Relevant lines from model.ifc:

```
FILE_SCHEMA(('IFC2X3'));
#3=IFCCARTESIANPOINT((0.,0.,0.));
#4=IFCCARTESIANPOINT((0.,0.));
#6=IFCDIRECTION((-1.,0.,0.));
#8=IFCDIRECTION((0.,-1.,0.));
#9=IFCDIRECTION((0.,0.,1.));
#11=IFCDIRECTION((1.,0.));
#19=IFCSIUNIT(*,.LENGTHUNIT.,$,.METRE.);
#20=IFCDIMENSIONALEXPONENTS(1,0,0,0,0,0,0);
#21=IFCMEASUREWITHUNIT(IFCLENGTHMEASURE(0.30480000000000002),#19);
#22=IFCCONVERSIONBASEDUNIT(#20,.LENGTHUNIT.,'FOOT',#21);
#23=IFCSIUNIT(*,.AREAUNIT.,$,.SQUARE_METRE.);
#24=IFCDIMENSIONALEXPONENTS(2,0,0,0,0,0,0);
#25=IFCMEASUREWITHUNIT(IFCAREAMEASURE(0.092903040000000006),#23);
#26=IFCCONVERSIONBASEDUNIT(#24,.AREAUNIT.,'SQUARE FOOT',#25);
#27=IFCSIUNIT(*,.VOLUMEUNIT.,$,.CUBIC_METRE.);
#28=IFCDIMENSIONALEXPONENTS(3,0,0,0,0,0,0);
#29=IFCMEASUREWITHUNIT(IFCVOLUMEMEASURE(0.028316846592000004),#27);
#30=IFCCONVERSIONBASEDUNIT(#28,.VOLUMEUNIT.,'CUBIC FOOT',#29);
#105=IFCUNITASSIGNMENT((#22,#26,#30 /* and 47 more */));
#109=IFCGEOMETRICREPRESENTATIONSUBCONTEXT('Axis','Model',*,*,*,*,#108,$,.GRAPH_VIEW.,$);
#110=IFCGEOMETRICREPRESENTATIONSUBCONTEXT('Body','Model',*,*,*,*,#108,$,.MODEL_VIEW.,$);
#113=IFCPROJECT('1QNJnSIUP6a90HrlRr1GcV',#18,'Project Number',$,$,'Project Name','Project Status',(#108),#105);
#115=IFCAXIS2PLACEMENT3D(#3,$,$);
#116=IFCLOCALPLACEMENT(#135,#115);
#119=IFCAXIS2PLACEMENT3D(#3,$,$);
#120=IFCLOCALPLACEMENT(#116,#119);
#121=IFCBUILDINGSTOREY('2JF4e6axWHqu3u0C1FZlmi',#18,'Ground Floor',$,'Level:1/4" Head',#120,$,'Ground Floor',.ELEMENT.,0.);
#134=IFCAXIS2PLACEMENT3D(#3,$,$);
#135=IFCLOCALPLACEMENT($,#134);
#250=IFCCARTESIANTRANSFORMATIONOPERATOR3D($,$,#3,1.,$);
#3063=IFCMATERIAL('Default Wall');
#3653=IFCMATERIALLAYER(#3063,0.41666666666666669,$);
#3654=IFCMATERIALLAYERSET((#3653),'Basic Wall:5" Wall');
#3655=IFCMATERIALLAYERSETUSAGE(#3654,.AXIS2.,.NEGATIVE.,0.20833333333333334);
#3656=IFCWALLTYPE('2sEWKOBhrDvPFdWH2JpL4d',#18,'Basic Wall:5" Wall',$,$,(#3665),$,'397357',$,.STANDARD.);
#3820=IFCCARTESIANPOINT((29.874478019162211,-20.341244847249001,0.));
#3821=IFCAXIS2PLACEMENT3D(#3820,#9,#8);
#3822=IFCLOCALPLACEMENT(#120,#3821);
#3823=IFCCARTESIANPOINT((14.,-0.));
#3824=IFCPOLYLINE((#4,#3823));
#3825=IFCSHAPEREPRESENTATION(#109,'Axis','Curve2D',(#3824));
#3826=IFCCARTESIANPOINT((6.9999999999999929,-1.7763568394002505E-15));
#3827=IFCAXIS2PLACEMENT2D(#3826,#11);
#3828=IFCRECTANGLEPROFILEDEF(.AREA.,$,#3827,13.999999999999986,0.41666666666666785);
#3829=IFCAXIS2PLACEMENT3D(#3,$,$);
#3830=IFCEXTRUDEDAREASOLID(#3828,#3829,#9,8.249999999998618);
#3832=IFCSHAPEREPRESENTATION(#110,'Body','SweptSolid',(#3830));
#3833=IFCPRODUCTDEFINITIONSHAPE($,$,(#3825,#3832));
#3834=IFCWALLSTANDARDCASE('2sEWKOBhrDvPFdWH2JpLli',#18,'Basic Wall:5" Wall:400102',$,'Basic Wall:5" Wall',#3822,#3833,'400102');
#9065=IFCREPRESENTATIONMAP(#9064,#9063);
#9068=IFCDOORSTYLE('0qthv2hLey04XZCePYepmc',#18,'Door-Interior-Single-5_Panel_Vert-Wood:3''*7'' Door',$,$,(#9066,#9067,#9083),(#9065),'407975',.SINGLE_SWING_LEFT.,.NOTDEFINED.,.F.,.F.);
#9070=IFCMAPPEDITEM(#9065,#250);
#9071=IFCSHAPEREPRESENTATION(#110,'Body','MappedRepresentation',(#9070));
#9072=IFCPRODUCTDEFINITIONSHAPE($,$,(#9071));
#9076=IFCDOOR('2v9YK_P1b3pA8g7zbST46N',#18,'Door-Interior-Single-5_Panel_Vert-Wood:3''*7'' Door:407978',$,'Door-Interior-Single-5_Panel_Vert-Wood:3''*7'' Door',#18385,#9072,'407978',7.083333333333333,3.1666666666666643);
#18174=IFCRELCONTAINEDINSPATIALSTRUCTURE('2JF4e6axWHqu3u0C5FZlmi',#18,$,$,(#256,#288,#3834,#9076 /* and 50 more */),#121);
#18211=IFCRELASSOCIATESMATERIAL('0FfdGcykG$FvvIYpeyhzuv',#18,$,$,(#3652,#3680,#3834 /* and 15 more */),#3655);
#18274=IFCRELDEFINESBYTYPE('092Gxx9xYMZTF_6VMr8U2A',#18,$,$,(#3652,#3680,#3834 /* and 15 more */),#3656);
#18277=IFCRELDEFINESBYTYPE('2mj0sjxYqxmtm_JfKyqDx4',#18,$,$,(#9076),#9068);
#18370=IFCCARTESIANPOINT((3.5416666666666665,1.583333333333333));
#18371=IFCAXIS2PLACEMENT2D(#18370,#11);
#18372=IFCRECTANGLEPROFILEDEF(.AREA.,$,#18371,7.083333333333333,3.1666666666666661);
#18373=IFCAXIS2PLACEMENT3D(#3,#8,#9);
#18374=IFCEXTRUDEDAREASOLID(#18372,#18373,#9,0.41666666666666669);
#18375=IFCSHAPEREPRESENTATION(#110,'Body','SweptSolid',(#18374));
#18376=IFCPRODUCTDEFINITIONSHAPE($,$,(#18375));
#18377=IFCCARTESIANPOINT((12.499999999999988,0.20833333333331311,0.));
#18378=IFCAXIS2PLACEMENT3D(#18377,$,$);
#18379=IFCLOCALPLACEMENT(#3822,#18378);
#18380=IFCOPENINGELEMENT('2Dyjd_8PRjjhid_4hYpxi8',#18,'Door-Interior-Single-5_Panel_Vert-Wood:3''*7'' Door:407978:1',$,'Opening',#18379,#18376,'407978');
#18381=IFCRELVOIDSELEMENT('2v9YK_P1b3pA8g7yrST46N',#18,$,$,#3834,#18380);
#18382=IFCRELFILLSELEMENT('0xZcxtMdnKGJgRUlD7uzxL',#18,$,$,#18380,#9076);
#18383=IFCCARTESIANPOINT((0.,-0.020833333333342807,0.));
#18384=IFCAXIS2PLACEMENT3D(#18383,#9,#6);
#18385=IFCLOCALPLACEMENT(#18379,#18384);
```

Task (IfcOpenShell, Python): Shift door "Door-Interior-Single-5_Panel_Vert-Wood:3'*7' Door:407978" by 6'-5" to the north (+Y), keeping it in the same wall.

```python
import ifcopenshell
import ifcopenshell.api.geometry
import ifcopenshell.util.placement
import ifcopenshell.util.unit

model = ifcopenshell.open("model.ifc")
unit_scale = ifcopenshell.util.unit.calculate_unit_scale(model)

door = model.by_guid("2v9YK_P1b3pA8g7zbST46N")
opening = door.FillsVoids[0].RelatingOpeningElement
wall = opening.VoidsElements[0].RelatingBuildingElement

wall_matrix = ifcopenshell.util.placement.get_local_placement(wall.ObjectPlacement)
shift = wall_matrix[:3, 0] * -77 * 0.0254 / unit_scale
before = ifcopenshell.util.placement.get_local_placement(door.ObjectPlacement)[:3, 3].copy()

# The door is placed relative to its opening, so it follows when the opening moves.
matrix = ifcopenshell.util.placement.get_local_placement(opening.ObjectPlacement)
matrix[:3, 3] += shift
ifcopenshell.api.geometry.edit_object_placement(
    model, product=opening, matrix=matrix, is_si=False, should_transform_children=True
)

after = ifcopenshell.util.placement.get_local_placement(door.ObjectPlacement)[:3, 3]
print("door moved by", (after - before).round(3) + 0.0)

model.write("model_rev.ifc")
```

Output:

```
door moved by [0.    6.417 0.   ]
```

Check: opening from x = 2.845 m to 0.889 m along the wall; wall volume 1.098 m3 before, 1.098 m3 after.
